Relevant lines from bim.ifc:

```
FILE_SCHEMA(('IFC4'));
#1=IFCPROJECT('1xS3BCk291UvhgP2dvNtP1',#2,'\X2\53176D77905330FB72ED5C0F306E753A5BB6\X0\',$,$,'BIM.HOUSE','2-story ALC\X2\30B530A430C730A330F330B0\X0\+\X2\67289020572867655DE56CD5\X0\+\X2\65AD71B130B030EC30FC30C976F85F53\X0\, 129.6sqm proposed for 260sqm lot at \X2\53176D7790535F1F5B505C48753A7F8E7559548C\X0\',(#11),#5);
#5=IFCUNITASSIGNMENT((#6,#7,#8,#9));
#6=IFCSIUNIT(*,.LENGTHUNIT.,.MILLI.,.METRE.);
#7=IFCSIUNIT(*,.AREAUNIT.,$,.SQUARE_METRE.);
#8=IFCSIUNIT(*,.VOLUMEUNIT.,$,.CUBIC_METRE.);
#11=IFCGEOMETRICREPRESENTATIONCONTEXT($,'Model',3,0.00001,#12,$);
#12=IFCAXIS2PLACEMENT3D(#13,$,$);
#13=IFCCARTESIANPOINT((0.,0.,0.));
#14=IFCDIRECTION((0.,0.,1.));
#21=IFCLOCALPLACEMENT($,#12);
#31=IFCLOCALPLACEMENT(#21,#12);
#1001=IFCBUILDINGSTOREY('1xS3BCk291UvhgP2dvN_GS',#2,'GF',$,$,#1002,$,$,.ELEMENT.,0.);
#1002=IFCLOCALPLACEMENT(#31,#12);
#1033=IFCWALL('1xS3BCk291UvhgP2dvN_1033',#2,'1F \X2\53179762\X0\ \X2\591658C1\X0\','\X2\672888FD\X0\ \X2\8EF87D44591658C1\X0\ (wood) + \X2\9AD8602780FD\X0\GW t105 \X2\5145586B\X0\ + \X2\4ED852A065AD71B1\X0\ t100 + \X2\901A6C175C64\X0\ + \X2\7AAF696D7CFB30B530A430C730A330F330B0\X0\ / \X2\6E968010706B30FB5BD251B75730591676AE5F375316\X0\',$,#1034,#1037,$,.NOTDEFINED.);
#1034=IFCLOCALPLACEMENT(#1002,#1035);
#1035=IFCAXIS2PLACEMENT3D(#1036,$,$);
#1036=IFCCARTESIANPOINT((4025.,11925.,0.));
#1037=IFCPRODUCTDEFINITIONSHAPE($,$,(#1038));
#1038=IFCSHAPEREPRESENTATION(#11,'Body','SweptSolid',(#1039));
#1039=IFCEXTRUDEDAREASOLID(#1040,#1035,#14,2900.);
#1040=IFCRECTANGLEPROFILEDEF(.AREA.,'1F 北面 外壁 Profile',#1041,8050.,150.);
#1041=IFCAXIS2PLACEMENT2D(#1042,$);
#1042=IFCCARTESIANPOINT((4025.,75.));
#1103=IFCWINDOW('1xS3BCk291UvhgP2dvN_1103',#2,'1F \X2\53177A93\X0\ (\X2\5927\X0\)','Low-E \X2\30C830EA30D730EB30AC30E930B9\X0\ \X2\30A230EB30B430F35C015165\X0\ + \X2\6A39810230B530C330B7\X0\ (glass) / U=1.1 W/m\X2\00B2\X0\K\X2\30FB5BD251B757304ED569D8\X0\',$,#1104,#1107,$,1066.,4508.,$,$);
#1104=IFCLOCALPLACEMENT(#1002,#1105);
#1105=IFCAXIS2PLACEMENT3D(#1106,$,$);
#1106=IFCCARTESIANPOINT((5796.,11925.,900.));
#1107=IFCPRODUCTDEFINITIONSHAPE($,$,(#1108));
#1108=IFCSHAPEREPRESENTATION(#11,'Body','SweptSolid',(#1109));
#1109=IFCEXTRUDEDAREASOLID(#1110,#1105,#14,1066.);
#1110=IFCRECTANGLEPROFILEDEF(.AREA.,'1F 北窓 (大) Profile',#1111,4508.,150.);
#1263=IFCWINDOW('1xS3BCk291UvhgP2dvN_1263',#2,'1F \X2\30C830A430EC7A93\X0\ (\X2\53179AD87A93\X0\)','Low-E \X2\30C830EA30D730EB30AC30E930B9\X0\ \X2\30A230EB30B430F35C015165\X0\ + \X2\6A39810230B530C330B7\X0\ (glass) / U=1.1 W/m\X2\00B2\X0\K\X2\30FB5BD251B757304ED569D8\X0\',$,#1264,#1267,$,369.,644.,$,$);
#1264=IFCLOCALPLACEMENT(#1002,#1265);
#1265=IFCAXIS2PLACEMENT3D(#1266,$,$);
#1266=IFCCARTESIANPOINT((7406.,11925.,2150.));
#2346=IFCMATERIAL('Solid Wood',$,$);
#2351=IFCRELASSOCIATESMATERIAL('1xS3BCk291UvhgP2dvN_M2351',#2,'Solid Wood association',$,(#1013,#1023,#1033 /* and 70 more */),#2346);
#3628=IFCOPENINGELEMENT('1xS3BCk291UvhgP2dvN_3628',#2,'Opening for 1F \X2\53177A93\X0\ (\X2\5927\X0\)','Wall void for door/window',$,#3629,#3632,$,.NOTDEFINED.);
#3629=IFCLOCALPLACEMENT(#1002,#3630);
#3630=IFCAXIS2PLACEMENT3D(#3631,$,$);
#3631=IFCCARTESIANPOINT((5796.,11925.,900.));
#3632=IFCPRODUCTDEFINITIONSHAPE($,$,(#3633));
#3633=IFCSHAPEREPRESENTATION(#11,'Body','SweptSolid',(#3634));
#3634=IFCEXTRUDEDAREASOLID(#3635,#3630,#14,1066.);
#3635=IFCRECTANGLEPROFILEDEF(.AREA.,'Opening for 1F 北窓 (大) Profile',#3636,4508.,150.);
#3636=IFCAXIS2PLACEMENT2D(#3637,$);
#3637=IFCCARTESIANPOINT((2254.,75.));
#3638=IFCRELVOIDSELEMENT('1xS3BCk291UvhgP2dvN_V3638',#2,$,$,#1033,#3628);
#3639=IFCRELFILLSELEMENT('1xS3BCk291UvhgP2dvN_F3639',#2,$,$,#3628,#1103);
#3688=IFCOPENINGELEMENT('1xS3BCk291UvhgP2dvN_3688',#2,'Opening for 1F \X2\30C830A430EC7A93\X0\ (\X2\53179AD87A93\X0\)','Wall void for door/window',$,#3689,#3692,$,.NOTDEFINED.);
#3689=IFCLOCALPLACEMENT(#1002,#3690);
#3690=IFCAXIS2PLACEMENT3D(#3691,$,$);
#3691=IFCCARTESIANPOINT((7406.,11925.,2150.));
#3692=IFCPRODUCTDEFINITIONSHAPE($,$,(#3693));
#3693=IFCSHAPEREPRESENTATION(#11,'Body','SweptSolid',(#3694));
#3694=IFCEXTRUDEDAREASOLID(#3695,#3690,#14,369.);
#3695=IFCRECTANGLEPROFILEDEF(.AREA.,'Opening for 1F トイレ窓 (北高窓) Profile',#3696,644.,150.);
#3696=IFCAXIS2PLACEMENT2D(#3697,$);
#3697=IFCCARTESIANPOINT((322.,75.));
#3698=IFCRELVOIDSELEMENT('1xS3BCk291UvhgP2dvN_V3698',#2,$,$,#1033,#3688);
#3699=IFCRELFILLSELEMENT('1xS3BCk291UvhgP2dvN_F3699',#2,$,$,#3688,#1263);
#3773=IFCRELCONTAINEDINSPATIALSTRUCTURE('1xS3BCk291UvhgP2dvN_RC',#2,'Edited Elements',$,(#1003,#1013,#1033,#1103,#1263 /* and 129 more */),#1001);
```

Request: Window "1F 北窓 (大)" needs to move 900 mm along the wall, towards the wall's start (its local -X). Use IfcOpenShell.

```python
import ifcopenshell
import ifcopenshell.api.geometry
import ifcopenshell.util.placement

model = ifcopenshell.open("bim.ifc")

window = model.by_guid("1xS3BCk291UvhgP2dvN_1103")
opening = window.FillsVoids[0].RelatingOpeningElement
wall = opening.VoidsElements[0].RelatingBuildingElement

wall_matrix = ifcopenshell.util.placement.get_local_placement(wall.ObjectPlacement)
shift = wall_matrix[:3, 0] * -900.0
before = ifcopenshell.util.placement.get_local_placement(window.ObjectPlacement)[:3, 3].copy()

# The window is not placed relative to its opening, so move both.
for product in (opening, window):
    matrix = ifcopenshell.util.placement.get_local_placement(product.ObjectPlacement)
    matrix[:3, 3] += shift
    ifcopenshell.api.geometry.edit_object_placement(model, product=product, matrix=matrix, is_si=False)

after = ifcopenshell.util.placement.get_local_placement(window.ObjectPlacement)[:3, 3]
print("window moved by", (after - before).round(3) + 0.0)

model.write("bim-out.ifc")
```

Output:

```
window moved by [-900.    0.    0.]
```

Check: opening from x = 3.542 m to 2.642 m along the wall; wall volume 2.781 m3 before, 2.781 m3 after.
